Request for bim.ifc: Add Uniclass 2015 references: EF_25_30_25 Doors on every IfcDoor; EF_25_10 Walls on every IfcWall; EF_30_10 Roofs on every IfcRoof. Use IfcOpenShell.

First a look at what the model holds.

```python
import ifcopenshell

model = ifcopenshell.open("bim.ifc")
print(model.schema)
print("classifications:", [c.Name for c in model.by_type("IfcClassification")])
for ifc_class in ("IfcDoor", "IfcRoof", "IfcStair", "IfcWall", "IfcWindow"):
    print(ifc_class, len(model.by_type(ifc_class)))
```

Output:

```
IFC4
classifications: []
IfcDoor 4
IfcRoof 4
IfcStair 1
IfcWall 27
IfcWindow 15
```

```python
import ifcopenshell
import ifcopenshell.api.classification

model = ifcopenshell.open("bim.ifc")

system = ifcopenshell.api.classification.add_classification(model, classification="Uniclass 2015")

codes = {
    "IfcDoor": ("EF_25_30_25", "Doors"),
    "IfcWall": ("EF_25_10", "Walls"),
    "IfcRoof": ("EF_30_10", "Roofs"),
}
for ifc_class, (code, name) in codes.items():
    products = model.by_type(ifc_class)
    ifcopenshell.api.classification.add_reference(
        model, products=products, classification=system, identification=code, name=name
    )
    print(code, len(products))

model.write("bim_edited.ifc")
```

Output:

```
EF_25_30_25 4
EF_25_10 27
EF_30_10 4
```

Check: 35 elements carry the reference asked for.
